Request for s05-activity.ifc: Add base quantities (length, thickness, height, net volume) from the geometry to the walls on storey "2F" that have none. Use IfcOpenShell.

First a look at what the model holds.

```python
import ifcopenshell
import ifcopenshell.util.element
import ifcopenshell.util.unit

model = ifcopenshell.open("s05-activity.ifc")
print(model.schema)
for unit_type in ("LENGTHUNIT", "AREAUNIT", "VOLUMEUNIT"):
    print(unit_type, ifcopenshell.util.unit.calculate_unit_scale(model, unit_type))
storey = next(s for s in model.by_type("IfcBuildingStorey") if s.Name == "2F")
walls = [e for e in ifcopenshell.util.element.get_decomposition(storey) if e.is_a("IfcWall")]
for e in sorted(walls, key=lambda e: e.id()):
    print(e.id(), e.is_a(), e.Name, list(ifcopenshell.util.element.get_psets(e, qtos_only=True)), sep=" | ")
```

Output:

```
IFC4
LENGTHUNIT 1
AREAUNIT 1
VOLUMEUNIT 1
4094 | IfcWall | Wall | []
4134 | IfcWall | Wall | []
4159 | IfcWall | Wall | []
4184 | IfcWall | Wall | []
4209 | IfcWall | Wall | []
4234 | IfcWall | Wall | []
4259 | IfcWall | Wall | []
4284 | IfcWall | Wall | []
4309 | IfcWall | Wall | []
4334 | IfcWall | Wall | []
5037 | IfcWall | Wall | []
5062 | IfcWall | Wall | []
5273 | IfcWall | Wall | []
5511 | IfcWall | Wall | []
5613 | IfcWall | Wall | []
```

```python
import ifcopenshell
import ifcopenshell.api.pset
import ifcopenshell.geom
import ifcopenshell.util.element
import ifcopenshell.util.shape
import ifcopenshell.util.unit

model = ifcopenshell.open("s05-activity.ifc")
unit_scale = ifcopenshell.util.unit.calculate_unit_scale(model)
volume_scale = ifcopenshell.util.unit.calculate_unit_scale(model, "VOLUMEUNIT")
settings = ifcopenshell.geom.settings()

storey = next(s for s in model.by_type("IfcBuildingStorey") if s.Name == "2F")
walls = [e for e in ifcopenshell.util.element.get_decomposition(storey) if e.is_a("IfcWall")]

for e in sorted(walls, key=lambda e: e.id()):
    if ifcopenshell.util.element.get_psets(e, qtos_only=True, should_inherit=False):
        continue
    # Geometry comes back in metres, in the element's own axes.
    shape = ifcopenshell.geom.create_shape(settings, e)
    values = {
        "Length": ifcopenshell.util.shape.get_x(shape.geometry) / unit_scale,
        "Width": ifcopenshell.util.shape.get_y(shape.geometry) / unit_scale,
        "Height": ifcopenshell.util.shape.get_z(shape.geometry) / unit_scale,
        "NetVolume": ifcopenshell.util.shape.get_volume(shape.geometry) / volume_scale,
    }
    qto = ifcopenshell.api.pset.add_qto(model, product=e, name="Qto_WallBaseQuantities")
    ifcopenshell.api.pset.edit_qto(model, qto=qto, properties=values)
    print(e.id(), {k: round(v, 3) for k, v in values.items()})

model.write("s05-activity_edited.ifc")
```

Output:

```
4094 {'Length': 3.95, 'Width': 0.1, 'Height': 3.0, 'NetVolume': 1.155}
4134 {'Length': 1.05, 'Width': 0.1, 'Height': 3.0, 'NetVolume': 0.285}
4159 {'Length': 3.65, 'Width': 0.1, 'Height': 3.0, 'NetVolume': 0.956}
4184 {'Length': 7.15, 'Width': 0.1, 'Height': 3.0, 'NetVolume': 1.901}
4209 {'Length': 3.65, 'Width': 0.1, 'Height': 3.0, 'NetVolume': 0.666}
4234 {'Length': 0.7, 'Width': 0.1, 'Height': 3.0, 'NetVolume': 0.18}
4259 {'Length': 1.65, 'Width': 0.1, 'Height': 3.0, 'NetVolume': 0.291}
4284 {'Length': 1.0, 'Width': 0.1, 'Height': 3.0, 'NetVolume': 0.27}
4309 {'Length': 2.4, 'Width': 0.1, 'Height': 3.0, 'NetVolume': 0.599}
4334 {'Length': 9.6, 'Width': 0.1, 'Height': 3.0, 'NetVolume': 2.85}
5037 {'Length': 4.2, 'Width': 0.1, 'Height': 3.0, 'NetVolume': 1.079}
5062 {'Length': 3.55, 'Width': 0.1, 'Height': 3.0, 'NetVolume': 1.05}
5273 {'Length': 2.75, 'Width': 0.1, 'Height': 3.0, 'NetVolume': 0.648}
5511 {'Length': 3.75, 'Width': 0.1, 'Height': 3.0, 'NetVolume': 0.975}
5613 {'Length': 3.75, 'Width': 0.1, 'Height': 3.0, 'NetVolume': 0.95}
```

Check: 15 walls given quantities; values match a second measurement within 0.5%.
